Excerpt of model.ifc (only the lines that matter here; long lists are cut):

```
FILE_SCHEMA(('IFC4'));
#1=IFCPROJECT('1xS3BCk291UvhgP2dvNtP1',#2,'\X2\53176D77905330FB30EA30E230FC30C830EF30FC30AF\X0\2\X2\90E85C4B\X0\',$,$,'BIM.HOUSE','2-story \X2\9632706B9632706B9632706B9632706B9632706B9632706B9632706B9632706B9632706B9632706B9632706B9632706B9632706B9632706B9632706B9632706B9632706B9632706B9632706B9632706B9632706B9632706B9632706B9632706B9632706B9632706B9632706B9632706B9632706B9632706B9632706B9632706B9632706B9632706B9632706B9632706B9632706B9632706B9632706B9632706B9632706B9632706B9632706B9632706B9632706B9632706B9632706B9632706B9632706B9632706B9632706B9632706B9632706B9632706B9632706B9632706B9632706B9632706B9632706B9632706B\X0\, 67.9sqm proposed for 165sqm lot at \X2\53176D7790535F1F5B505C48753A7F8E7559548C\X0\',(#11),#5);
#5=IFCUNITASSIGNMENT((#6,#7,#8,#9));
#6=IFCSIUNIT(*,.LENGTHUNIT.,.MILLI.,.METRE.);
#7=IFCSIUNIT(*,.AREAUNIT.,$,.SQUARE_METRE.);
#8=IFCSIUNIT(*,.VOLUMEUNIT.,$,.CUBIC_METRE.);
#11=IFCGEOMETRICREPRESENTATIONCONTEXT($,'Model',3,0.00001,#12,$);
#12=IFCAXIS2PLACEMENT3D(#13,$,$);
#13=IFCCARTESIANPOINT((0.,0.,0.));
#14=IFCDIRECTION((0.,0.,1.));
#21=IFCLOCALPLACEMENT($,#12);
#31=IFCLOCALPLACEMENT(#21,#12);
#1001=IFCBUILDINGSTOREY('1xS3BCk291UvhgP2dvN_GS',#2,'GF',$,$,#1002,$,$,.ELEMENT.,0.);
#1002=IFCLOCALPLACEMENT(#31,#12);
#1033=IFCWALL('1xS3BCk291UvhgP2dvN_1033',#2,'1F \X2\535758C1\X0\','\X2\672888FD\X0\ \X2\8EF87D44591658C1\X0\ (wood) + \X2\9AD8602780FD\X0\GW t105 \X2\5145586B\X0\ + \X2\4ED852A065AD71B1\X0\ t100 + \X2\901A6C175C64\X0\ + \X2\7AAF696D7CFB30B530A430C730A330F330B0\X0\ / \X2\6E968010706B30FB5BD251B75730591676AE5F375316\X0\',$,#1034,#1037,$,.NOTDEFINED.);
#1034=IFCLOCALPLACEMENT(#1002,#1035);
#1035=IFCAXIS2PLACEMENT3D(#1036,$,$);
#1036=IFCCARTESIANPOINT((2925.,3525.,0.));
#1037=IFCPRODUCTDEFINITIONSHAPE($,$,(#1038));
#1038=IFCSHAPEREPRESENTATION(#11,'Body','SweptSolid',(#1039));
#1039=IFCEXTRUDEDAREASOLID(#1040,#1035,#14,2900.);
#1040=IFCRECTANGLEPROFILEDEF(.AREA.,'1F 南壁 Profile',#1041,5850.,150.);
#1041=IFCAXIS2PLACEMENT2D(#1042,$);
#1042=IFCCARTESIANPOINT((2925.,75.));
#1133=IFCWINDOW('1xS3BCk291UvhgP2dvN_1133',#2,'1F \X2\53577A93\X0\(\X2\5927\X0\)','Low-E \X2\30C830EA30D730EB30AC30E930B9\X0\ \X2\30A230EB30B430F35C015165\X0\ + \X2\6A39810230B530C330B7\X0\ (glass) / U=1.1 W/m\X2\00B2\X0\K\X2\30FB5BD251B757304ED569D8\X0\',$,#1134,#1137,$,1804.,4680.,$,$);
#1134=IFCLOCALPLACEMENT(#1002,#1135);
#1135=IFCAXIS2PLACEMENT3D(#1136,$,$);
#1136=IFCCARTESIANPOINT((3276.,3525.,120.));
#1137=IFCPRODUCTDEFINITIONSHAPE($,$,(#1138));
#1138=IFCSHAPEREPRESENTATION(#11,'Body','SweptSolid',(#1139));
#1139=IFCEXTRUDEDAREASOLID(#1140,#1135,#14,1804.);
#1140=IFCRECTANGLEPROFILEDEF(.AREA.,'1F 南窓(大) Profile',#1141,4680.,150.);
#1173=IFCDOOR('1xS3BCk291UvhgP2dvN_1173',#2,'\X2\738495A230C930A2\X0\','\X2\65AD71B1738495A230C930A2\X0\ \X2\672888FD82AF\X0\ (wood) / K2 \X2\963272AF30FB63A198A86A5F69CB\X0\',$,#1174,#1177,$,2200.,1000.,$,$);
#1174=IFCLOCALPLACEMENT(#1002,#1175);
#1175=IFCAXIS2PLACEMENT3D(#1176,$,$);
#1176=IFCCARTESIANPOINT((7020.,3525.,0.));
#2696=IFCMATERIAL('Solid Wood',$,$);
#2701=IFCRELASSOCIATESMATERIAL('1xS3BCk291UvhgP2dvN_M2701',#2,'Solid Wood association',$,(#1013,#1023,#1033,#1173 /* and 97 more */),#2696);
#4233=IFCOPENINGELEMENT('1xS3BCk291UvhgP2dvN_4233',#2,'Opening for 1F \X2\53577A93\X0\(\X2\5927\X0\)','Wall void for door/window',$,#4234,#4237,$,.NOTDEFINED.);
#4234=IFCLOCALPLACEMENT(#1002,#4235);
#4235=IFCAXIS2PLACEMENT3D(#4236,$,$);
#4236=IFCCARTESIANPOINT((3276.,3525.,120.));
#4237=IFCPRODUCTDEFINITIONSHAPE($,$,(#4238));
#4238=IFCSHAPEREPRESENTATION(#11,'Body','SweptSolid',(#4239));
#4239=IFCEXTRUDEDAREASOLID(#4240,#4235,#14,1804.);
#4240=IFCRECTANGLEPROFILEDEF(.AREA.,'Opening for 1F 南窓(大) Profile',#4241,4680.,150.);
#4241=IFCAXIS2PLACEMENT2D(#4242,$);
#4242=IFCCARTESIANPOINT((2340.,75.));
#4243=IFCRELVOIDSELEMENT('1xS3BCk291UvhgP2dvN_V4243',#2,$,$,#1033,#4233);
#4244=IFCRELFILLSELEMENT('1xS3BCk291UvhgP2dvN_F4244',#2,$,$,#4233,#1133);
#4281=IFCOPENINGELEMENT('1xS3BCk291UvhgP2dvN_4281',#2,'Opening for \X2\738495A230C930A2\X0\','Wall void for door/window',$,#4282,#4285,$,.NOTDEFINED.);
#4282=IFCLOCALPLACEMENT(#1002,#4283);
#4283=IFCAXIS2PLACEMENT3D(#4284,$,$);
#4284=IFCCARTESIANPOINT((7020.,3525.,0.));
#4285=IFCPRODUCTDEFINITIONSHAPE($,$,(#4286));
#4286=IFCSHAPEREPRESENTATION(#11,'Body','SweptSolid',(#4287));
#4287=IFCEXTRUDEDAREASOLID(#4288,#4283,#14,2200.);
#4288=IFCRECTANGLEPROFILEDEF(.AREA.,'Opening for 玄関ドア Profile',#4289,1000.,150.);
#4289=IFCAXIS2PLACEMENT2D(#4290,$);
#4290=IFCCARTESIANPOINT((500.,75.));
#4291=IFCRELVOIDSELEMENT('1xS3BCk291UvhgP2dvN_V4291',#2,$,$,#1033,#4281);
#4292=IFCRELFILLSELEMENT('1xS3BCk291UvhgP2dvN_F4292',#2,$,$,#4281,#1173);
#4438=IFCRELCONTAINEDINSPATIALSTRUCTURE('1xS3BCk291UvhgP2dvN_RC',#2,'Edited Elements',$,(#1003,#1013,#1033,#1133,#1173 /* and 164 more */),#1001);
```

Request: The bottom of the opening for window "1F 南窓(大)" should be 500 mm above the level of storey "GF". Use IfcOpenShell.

```python
import numpy as np
import ifcopenshell
import ifcopenshell.api.geometry
import ifcopenshell.geom
import ifcopenshell.util.element
import ifcopenshell.util.placement
import ifcopenshell.util.shape
import ifcopenshell.util.unit

model = ifcopenshell.open("model.ifc")
unit_scale = ifcopenshell.util.unit.calculate_unit_scale(model)

window = model.by_id(1133)
opening = window.FillsVoids[0].RelatingOpeningElement
storey = ifcopenshell.util.element.get_container(window, ifc_class="IfcBuildingStorey")
level = ifcopenshell.util.placement.get_local_placement(storey.ObjectPlacement)[2, 3]

# The opening's origin need not be at the sill, so measure its lowest point.
shape = ifcopenshell.geom.create_shape(ifcopenshell.geom.settings(), opening)
bottom = ifcopenshell.util.shape.get_shape_bottom_elevation(shape, shape.geometry) / unit_scale
dz = level + 0.5 / unit_scale - bottom

shift = np.array([0.0, 0.0, dz])
# The window is not placed relative to its opening, so move both.
for product in (opening, window):
    matrix = ifcopenshell.util.placement.get_local_placement(product.ObjectPlacement)
    matrix[:3, 3] += shift
    ifcopenshell.api.geometry.edit_object_placement(model, product=product, matrix=matrix, is_si=False)

print(f"moved by {dz * unit_scale:+.3f} m")

model.write("model-out.ifc")
```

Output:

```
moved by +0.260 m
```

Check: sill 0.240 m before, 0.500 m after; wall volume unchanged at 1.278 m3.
